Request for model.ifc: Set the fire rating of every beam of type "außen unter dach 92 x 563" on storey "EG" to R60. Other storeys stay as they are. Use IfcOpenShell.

First a look at what the model holds.

```python
import ifcopenshell
import ifcopenshell.util.element

model = ifcopenshell.open("model.ifc")
print(model.schema)
storey = next(s for s in model.by_type("IfcBuildingStorey") if s.Name == "EG")
beams = [e for e in ifcopenshell.util.element.get_decomposition(storey) if e.is_a("IfcBeam")]
seen = {}
for e in beams:
    element_type = ifcopenshell.util.element.get_type(e)
    key = (element_type.Name if element_type != e and element_type else None, ifcopenshell.util.element.get_pset(e, "Pset_BeamCommon", "FireRating"))
    seen[key] = seen.get(key, 0) + 1
for (name, value), count in sorted(seen.items(), key=str):
    print(count, "x", name, "|", value)
```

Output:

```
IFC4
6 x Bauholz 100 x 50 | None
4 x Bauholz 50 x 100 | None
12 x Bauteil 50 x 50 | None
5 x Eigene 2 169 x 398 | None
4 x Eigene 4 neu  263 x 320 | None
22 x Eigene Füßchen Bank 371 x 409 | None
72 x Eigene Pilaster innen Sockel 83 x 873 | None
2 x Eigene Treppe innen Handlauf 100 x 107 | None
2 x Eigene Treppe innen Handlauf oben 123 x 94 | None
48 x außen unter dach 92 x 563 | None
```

```python
import ifcopenshell
import ifcopenshell.api.pset
import ifcopenshell.util.element

model = ifcopenshell.open("model.ifc")

storey = next(s for s in model.by_type("IfcBuildingStorey") if s.Name == "EG")
beams = [e for e in ifcopenshell.util.element.get_decomposition(storey) if e.is_a("IfcBeam")]

count = 0
for e in beams:
    element_type = ifcopenshell.util.element.get_type(e)
    if element_type in (None, e) or element_type.Name != "außen unter dach 92 x 563":
        continue
    # add_pset returns the element's existing set when there is one.
    pset = ifcopenshell.api.pset.add_pset(model, product=e, name="Pset_BeamCommon")
    ifcopenshell.api.pset.edit_pset(model, pset=pset, properties={"FireRating": "R60"})
    count += 1

print(count, "beams updated")

model.write("model_rev.ifc")
```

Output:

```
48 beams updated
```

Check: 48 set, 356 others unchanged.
